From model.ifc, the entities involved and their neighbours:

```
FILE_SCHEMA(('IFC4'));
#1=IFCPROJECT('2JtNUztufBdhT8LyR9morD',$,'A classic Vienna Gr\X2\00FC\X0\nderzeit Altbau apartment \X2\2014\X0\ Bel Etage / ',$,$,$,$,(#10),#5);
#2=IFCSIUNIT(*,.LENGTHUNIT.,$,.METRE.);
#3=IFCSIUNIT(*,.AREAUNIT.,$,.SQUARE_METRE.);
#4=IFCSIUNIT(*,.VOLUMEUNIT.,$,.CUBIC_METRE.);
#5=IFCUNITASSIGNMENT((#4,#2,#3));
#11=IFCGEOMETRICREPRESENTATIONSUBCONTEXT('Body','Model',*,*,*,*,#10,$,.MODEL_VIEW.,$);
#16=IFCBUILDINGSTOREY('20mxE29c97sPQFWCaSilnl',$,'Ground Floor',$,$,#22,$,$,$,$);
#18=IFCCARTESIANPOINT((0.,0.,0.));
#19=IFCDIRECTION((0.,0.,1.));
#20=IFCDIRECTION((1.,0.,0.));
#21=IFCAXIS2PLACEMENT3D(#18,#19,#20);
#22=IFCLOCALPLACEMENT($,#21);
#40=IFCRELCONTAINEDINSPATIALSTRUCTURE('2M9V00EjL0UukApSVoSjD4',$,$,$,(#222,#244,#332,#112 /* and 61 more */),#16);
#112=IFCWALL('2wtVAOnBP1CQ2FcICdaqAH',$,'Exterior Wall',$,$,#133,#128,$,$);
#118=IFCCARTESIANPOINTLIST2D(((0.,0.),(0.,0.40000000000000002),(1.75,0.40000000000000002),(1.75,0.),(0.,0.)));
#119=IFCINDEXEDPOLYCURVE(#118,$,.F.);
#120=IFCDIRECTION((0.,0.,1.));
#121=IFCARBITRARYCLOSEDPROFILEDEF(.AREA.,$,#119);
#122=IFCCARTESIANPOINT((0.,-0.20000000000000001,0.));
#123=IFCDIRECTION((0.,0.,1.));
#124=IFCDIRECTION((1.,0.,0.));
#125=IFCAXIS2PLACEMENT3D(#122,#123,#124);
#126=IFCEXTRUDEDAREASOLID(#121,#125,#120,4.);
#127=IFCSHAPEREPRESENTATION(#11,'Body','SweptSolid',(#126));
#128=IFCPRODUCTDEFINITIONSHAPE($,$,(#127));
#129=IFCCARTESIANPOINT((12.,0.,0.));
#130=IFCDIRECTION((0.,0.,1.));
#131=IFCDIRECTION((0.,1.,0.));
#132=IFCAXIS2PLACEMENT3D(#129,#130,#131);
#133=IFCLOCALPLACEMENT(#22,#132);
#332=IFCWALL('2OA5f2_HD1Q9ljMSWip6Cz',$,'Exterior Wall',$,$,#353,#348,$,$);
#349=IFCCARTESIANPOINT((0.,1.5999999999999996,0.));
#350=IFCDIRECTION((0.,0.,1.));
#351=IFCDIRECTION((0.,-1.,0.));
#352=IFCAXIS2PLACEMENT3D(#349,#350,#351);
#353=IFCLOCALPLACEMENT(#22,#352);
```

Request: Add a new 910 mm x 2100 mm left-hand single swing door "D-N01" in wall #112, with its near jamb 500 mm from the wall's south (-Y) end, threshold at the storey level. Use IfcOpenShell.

```python
import numpy as np
import ifcopenshell
import ifcopenshell.api.feature
import ifcopenshell.api.geometry
import ifcopenshell.api.root
import ifcopenshell.api.spatial
import ifcopenshell.geom
import ifcopenshell.util.element
import ifcopenshell.util.placement
import ifcopenshell.util.representation
import ifcopenshell.util.shape
import ifcopenshell.util.unit

model = ifcopenshell.open("model.ifc")
unit_scale = ifcopenshell.util.unit.calculate_unit_scale(model)
settings = ifcopenshell.geom.settings()


def volume(element):
    """Net volume in cubic metres, openings subtracted."""
    shape = ifcopenshell.geom.create_shape(settings, element)
    return ifcopenshell.util.shape.get_volume(shape.geometry)


wall = model.by_id(112)
storey = ifcopenshell.util.element.get_container(wall, ifc_class="IfcBuildingStorey")
context = ifcopenshell.util.representation.get_context(model, "Model", "Body", "MODEL_VIEW")
before = volume(wall)

width, height, from_end, sill = 0.91, 2.1, 0.5, 0.0  # metres

# The wall runs along its own X axis, and the end named is its -X end.
wall_shape = ifcopenshell.geom.create_shape(settings, wall)
x, y, z = ifcopenshell.util.shape.get_vertices(wall_shape.geometry).T
start = x.min() + from_end
face, thickness = float(y.min()), float(y.max() - y.min())
wall_matrix = ifcopenshell.util.placement.get_local_placement(wall.ObjectPlacement)
level = ifcopenshell.util.placement.get_local_placement(storey.ObjectPlacement)[2, 3]


def in_wall(x, y):
    """Placement at x, y metres in the wall's axes, at sill height."""
    matrix = wall_matrix.copy()
    matrix[:, 3] = wall_matrix @ np.array([x / unit_scale, y / unit_scale, 0.0, 1.0])
    matrix[2, 3] = level + sill / unit_scale
    return matrix


# Opening: a box that overshoots both wall faces by 50 mm.
opening = ifcopenshell.api.root.create_entity(model, ifc_class="IfcOpeningElement", predefined_type="OPENING")
box = ifcopenshell.api.geometry.add_wall_representation(
    model, context=context, length=width, height=height, thickness=thickness + 0.1
)
ifcopenshell.api.geometry.assign_representation(model, product=opening, representation=box)
ifcopenshell.api.geometry.edit_object_placement(model, product=opening, matrix=in_wall(start, face - 0.05), is_si=False)
ifcopenshell.api.feature.add_feature(model, feature=opening, element=wall)

door = ifcopenshell.api.root.create_entity(model, ifc_class="IfcDoor", name="D-N01", predefined_type="DOOR")
door.OverallWidth, door.OverallHeight = width / unit_scale, height / unit_scale
door.OperationType = "SINGLE_SWING_LEFT"
body = ifcopenshell.api.geometry.add_door_representation(
    model,
    context=context,
    overall_width=door.OverallWidth,
    overall_height=door.OverallHeight,
    operation_type="SINGLE_SWING_LEFT",
    lining_properties={"LiningDepth": thickness / unit_scale, "ThresholdDepth": thickness / unit_scale},
)
ifcopenshell.api.geometry.assign_representation(model, product=door, representation=body)
ifcopenshell.api.spatial.assign_container(model, products=[door], relating_structure=storey)
ifcopenshell.api.feature.add_filling(model, opening=opening, element=door)

# The lining spans the wall, so the door starts at the wall face.
ifcopenshell.api.geometry.edit_object_placement(model, product=door, matrix=in_wall(start, face), is_si=False)

after = volume(wall)

print(f"wall volume {before:.3f} -> {after:.3f} m3")

model.write("model_v2.ifc")
```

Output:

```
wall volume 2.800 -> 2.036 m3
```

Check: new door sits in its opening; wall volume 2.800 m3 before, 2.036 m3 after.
